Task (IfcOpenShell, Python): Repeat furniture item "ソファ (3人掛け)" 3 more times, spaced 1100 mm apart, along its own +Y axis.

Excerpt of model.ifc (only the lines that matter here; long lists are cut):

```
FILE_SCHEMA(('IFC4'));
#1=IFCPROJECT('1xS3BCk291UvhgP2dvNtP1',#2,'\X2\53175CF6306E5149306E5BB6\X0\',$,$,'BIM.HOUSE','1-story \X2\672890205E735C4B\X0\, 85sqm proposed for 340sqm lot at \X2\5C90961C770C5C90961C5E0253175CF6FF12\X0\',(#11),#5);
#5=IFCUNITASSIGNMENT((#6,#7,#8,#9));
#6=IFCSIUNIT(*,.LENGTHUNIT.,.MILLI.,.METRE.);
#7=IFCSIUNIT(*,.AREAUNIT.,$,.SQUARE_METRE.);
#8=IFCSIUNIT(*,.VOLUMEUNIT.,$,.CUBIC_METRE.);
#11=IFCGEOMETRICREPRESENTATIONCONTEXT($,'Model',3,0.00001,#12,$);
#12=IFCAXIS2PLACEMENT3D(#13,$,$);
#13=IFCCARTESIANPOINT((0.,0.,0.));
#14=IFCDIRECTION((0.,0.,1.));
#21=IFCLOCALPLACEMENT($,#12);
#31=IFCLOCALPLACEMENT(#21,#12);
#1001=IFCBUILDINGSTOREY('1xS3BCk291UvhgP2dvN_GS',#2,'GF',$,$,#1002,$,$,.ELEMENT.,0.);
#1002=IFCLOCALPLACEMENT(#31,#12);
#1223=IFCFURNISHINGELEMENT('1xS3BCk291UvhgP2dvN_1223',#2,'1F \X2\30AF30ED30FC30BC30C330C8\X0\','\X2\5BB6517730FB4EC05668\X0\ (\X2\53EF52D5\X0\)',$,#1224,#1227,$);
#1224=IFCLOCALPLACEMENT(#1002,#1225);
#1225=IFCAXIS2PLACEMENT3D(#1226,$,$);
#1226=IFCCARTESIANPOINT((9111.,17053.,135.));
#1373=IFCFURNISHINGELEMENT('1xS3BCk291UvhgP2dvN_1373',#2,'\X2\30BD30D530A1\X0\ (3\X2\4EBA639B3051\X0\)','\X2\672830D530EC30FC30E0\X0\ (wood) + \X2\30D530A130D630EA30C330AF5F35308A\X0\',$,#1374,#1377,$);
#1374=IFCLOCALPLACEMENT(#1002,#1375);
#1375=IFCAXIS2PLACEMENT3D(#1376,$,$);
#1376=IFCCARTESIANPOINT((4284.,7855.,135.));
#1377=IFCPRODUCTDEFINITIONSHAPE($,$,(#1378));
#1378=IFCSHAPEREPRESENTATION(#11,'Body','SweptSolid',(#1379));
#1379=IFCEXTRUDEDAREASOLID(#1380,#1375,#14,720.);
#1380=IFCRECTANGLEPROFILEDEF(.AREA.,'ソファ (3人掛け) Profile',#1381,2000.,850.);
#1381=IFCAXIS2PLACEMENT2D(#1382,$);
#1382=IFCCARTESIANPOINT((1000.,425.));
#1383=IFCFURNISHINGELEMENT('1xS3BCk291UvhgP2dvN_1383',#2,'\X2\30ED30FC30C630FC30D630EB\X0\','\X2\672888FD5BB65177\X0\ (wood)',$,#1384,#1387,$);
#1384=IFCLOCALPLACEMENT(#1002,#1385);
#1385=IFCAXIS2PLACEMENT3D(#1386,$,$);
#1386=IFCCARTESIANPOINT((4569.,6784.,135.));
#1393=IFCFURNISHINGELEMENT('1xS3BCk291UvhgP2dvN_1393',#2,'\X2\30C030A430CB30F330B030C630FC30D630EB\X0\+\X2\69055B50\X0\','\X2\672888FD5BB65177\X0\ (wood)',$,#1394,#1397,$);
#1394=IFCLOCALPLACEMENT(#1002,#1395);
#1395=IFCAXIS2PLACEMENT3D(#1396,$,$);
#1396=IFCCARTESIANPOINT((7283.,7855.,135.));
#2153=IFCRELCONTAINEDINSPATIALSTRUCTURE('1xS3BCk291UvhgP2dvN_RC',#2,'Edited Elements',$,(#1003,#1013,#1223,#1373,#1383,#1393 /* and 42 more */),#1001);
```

```python
import ifcopenshell
import ifcopenshell.api.geometry
import ifcopenshell.api.root
import ifcopenshell.util.element
import ifcopenshell.util.placement

model = ifcopenshell.open("model.ifc")


def reuse_history(source, copy):
    """copy_class also copies each property set's owner history, people and application; keep the originals."""
    for rel in copy.IsDefinedBy:
        if rel.is_a("IfcRelDefinesByProperties") and (history := rel.RelatingPropertyDefinition.OwnerHistory):
            rel.RelatingPropertyDefinition.OwnerHistory = source.OwnerHistory
            ifcopenshell.util.element.remove_deep2(model, history)


source = model.by_id(1373)
base = ifcopenshell.util.placement.get_local_placement(source.ObjectPlacement)
step = base[:3, 1] * 1100.0

for i in range(1, 4):
    copy = ifcopenshell.api.root.copy_class(model, product=source)
    copy.Representation = ifcopenshell.util.element.copy_deep(
        model, source.Representation, exclude=["IfcGeometricRepresentationContext", "IfcRepresentationMap"]
    )
    reuse_history(source, copy)
    matrix = base.copy()
    matrix[:3, 3] += i * step
    print("added at", matrix[:3, 3].round(3) + 0.0)
    ifcopenshell.api.geometry.edit_object_placement(model, product=copy, matrix=matrix, is_si=False)

model.write("model-out.ifc")
```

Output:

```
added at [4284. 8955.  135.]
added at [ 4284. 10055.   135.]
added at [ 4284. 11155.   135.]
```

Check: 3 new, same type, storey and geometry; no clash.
